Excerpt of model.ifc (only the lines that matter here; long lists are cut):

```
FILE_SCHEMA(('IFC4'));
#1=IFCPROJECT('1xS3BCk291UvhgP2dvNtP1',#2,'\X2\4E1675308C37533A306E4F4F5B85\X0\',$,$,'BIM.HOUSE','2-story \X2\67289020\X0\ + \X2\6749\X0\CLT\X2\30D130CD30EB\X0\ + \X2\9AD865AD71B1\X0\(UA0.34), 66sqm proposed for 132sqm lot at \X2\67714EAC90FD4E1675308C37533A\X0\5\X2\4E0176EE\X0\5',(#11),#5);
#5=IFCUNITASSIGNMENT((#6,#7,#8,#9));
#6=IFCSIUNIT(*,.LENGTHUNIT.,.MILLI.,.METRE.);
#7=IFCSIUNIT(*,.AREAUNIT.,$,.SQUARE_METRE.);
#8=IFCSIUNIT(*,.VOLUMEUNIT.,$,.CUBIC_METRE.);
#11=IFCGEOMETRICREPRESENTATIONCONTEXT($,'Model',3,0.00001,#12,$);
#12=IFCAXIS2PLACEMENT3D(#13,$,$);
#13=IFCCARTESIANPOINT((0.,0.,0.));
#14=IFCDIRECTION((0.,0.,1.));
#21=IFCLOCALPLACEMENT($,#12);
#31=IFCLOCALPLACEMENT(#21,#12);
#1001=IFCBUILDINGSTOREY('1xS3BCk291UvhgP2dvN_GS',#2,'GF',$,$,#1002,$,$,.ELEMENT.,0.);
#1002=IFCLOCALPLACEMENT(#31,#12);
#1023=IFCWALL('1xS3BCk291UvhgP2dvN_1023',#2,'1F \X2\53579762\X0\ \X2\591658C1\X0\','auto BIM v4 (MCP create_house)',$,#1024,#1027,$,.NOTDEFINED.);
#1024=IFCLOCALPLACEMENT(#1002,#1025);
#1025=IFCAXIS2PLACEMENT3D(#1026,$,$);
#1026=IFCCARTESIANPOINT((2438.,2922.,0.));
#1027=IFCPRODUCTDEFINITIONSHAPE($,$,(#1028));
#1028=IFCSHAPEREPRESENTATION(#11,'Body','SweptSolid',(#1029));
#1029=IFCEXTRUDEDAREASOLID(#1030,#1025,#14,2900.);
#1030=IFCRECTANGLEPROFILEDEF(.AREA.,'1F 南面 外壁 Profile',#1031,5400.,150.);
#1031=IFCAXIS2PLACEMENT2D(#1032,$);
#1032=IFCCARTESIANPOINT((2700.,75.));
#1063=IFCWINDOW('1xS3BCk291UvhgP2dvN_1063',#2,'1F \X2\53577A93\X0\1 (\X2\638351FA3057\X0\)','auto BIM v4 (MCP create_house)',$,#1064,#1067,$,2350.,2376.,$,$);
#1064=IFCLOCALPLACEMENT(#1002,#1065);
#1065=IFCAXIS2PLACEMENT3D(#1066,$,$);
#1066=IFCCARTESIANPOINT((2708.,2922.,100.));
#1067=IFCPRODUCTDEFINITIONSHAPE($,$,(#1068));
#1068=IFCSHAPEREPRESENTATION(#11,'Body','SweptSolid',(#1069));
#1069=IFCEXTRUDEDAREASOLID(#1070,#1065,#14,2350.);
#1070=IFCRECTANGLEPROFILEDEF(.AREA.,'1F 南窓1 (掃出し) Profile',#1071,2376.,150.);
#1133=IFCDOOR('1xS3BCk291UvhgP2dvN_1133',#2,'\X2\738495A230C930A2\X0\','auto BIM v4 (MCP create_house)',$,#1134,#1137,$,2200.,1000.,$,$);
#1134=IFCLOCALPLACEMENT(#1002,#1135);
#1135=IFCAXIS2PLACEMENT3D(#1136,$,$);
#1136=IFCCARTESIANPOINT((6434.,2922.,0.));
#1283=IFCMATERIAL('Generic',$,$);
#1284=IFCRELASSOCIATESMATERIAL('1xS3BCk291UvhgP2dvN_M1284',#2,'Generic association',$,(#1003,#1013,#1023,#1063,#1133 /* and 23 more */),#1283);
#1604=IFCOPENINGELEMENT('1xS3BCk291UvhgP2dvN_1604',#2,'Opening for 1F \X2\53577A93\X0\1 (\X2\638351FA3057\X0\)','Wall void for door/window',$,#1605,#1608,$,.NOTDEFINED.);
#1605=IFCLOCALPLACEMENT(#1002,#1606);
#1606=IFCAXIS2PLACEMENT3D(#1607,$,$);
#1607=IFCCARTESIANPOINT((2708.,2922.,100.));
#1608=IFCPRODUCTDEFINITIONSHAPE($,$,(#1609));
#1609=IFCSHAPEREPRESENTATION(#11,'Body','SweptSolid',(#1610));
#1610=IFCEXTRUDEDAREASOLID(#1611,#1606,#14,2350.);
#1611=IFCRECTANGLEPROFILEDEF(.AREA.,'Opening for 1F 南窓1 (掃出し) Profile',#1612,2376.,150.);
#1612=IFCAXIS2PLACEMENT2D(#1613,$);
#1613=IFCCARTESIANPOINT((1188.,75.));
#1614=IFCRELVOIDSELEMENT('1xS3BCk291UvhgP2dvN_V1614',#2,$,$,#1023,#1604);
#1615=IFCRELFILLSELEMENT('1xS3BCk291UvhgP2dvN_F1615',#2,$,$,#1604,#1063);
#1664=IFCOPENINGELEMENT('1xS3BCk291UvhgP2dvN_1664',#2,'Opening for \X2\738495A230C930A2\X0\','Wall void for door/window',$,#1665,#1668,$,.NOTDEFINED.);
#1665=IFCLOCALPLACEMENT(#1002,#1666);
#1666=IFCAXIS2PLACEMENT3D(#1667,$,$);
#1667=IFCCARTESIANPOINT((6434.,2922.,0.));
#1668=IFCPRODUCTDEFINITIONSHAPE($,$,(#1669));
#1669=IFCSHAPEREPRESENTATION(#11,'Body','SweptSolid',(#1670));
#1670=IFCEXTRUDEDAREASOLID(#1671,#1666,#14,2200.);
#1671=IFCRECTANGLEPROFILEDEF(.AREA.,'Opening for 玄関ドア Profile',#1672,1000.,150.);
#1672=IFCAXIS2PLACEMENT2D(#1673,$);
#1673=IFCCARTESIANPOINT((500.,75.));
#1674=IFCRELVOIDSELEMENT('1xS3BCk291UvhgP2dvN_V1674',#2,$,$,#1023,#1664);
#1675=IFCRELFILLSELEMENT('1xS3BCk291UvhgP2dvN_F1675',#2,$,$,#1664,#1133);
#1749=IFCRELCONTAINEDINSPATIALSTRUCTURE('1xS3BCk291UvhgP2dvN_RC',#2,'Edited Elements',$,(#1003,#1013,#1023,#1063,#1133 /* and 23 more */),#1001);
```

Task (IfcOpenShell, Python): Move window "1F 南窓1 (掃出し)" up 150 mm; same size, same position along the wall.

```python
import numpy as np
import ifcopenshell
import ifcopenshell.api.geometry
import ifcopenshell.util.placement
import ifcopenshell.util.unit

model = ifcopenshell.open("model.ifc")
unit_scale = ifcopenshell.util.unit.calculate_unit_scale(model)

window = model.by_guid("1xS3BCk291UvhgP2dvN_1063")
opening = window.FillsVoids[0].RelatingOpeningElement
dz = 0.15 / unit_scale

shift = np.array([0.0, 0.0, dz])
# The window is not placed relative to its opening, so move both.
for product in (opening, window):
    matrix = ifcopenshell.util.placement.get_local_placement(product.ObjectPlacement)
    matrix[:3, 3] += shift
    ifcopenshell.api.geometry.edit_object_placement(model, product=product, matrix=matrix, is_si=False)

print(f"moved by {dz * unit_scale:+.3f} m")

model.write("model_updated.ifc")
```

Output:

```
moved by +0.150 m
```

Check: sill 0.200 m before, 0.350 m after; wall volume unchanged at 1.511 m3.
